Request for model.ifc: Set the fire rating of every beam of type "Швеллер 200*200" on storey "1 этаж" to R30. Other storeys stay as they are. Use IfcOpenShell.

First a look at what the model holds.

```python
import ifcopenshell
import ifcopenshell.util.element

model = ifcopenshell.open("model.ifc")
print(model.schema)
storey = next(s for s in model.by_type("IfcBuildingStorey") if s.Name == "1 этаж")
beams = [e for e in ifcopenshell.util.element.get_decomposition(storey) if e.is_a("IfcBeam")]
seen = {}
for e in beams:
    element_type = ifcopenshell.util.element.get_type(e)
    key = (element_type.Name if element_type != e and element_type else None, ifcopenshell.util.element.get_pset(e, "Pset_BeamCommon", "FireRating"))
    seen[key] = seen.get(key, 0) + 1
for (name, value), count in sorted(seen.items(), key=str):
    print(count, "x", name, "|", value)
```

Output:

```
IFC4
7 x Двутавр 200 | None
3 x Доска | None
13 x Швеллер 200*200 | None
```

```python
import ifcopenshell
import ifcopenshell.api.pset
import ifcopenshell.util.element

model = ifcopenshell.open("model.ifc")

storey = next(s for s in model.by_type("IfcBuildingStorey") if s.Name == "1 этаж")
beams = [e for e in ifcopenshell.util.element.get_decomposition(storey) if e.is_a("IfcBeam")]

count = 0
for e in beams:
    element_type = ifcopenshell.util.element.get_type(e)
    if element_type in (None, e) or element_type.Name != "Швеллер 200*200":
        continue
    # add_pset returns the element's existing set when there is one.
    pset = ifcopenshell.api.pset.add_pset(model, product=e, name="Pset_BeamCommon")
    ifcopenshell.api.pset.edit_pset(model, pset=pset, properties={"FireRating": "R30"})
    count += 1

print(count, "beams updated")

model.write("model-out.ifc")
```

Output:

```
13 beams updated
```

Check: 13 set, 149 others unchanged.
